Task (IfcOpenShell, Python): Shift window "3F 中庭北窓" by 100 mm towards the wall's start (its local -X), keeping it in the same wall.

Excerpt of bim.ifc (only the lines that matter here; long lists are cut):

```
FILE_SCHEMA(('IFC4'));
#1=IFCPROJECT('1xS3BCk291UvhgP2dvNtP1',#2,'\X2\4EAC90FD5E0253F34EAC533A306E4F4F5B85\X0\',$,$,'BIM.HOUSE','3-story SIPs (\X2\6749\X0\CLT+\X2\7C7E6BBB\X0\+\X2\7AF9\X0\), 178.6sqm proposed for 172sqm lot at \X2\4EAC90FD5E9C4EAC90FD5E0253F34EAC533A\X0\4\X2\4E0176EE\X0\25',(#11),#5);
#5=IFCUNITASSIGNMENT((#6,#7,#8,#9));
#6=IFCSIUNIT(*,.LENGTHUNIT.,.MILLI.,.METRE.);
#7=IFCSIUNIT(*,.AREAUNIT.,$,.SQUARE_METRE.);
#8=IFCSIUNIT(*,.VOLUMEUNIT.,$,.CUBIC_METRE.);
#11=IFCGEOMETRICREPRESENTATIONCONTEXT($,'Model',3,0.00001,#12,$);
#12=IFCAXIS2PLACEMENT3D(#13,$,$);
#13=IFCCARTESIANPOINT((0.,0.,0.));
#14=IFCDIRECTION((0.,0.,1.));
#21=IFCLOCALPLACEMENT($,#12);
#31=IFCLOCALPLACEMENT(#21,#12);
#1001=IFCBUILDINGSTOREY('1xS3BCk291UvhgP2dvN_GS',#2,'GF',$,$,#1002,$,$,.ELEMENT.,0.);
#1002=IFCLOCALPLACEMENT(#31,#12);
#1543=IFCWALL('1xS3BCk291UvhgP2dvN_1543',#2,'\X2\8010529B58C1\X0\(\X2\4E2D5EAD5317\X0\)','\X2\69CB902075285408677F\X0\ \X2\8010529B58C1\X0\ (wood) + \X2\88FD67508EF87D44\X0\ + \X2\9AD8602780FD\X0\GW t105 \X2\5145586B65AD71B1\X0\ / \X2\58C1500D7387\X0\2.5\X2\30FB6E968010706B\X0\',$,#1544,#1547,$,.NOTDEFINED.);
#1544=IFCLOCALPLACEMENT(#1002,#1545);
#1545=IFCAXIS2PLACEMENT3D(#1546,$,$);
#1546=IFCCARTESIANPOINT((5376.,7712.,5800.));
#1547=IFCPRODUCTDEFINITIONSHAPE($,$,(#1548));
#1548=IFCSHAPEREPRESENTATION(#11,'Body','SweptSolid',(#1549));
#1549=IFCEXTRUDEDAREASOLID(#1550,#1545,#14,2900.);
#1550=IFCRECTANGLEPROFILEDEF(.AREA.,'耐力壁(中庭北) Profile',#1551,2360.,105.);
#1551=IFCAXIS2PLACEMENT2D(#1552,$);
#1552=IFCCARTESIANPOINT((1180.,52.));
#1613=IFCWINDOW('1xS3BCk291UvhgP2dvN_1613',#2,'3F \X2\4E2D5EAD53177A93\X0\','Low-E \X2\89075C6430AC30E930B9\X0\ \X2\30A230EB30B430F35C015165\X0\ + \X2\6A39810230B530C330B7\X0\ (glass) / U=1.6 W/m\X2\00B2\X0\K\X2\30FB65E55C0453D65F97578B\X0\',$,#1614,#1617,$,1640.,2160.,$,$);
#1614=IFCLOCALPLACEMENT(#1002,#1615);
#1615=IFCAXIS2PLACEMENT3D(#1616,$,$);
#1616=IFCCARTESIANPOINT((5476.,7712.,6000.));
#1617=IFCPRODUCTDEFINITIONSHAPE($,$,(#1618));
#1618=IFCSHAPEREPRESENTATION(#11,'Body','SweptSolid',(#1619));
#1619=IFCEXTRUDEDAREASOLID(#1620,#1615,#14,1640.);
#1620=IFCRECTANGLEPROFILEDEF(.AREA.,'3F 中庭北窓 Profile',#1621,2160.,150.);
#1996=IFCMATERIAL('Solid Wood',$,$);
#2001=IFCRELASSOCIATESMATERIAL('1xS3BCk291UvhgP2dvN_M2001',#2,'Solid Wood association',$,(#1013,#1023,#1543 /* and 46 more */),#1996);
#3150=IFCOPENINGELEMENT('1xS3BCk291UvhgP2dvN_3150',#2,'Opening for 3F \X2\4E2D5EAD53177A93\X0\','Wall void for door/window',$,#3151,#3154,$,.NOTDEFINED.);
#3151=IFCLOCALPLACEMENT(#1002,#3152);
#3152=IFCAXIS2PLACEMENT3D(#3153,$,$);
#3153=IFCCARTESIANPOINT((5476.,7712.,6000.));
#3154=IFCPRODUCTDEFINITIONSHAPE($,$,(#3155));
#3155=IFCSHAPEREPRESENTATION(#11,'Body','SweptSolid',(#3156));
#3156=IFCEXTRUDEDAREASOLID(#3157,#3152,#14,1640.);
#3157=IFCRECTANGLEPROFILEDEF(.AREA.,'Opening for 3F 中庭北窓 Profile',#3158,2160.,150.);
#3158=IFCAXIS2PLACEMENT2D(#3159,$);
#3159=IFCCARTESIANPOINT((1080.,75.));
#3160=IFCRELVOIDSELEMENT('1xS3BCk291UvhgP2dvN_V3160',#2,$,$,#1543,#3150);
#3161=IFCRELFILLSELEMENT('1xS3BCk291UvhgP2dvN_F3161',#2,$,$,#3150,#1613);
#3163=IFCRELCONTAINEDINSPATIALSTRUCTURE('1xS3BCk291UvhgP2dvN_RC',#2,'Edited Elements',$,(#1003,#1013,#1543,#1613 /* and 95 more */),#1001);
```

```python
import ifcopenshell
import ifcopenshell.api.geometry
import ifcopenshell.util.placement

model = ifcopenshell.open("bim.ifc")

window = model.by_guid("1xS3BCk291UvhgP2dvN_1613")
opening = window.FillsVoids[0].RelatingOpeningElement
wall = opening.VoidsElements[0].RelatingBuildingElement

wall_matrix = ifcopenshell.util.placement.get_local_placement(wall.ObjectPlacement)
shift = wall_matrix[:3, 0] * -100.0
before = ifcopenshell.util.placement.get_local_placement(window.ObjectPlacement)[:3, 3].copy()

# The window is not placed relative to its opening, so move both.
for product in (opening, window):
    matrix = ifcopenshell.util.placement.get_local_placement(product.ObjectPlacement)
    matrix[:3, 3] += shift
    ifcopenshell.api.geometry.edit_object_placement(model, product=product, matrix=matrix, is_si=False)

after = ifcopenshell.util.placement.get_local_placement(window.ObjectPlacement)[:3, 3]
print("window moved by", (after - before).round(3) + 0.0)

model.write("bim_updated.ifc")
```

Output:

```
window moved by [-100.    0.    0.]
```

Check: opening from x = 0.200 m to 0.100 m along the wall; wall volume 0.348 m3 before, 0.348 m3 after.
